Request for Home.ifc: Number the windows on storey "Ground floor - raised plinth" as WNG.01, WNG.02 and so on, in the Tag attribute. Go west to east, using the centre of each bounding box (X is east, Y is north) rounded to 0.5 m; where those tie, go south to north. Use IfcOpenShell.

First a look at what the model holds.

```python
import ifcopenshell
import ifcopenshell.util.element
import ifcopenshell.util.placement

model = ifcopenshell.open("Home.ifc")
print(model.schema)
storey = next(s for s in model.by_type("IfcBuildingStorey") if s.Name == "Ground floor - raised plinth")
windows = [e for e in ifcopenshell.util.element.get_decomposition(storey) if e.is_a("IfcWindow")]
for e in sorted(windows, key=lambda e: e.id()):
    origin = ifcopenshell.util.placement.get_local_placement(e.ObjectPlacement)[:3, 3]
    print(e.id(), e.Tag, e.Name, origin.round(2) + 0.0, sep=" | ")
```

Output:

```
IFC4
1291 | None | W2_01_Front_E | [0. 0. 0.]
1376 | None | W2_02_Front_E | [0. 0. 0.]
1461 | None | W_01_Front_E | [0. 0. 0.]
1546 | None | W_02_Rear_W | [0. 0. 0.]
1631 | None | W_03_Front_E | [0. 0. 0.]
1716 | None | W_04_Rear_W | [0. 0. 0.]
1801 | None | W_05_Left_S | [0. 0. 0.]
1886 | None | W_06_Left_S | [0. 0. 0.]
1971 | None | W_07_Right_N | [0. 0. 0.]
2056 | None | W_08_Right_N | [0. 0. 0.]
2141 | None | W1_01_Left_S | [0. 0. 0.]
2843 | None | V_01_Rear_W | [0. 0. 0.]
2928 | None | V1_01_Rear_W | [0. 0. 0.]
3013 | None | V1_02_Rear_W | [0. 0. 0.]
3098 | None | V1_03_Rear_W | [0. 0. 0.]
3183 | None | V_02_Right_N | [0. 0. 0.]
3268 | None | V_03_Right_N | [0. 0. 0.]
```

```python
import ifcopenshell
import ifcopenshell.geom
import ifcopenshell.util.element
import ifcopenshell.util.shape

model = ifcopenshell.open("Home.ifc")
settings = ifcopenshell.geom.settings()
settings.set("use-world-coords", True)


def centre(element):
    shape = ifcopenshell.geom.create_shape(settings, element)
    return ifcopenshell.util.shape.get_bbox_centroid(shape.geometry)


storey = next(s for s in model.by_type("IfcBuildingStorey") if s.Name == "Ground floor - raised plinth")
windows = [e for e in ifcopenshell.util.element.get_decomposition(storey) if e.is_a("IfcWindow")]

# Insertion points can sit at a corner or the storey origin, so sort by the geometry (in metres).
centres = {e: centre(e) for e in windows}
windows.sort(key=lambda e: (round(centres[e][0] / 0.5), centres[e][1]))

for i, e in enumerate(windows, start=1):
    number = f"WNG.{i:02d}"
    e.Tag = number
    print(e.id(), number)

model.write("Home-out.ifc")
```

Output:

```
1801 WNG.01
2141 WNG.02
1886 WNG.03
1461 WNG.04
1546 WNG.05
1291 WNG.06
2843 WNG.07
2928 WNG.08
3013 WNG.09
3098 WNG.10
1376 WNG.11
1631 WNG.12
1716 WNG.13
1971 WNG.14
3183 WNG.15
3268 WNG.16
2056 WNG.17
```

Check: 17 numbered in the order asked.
